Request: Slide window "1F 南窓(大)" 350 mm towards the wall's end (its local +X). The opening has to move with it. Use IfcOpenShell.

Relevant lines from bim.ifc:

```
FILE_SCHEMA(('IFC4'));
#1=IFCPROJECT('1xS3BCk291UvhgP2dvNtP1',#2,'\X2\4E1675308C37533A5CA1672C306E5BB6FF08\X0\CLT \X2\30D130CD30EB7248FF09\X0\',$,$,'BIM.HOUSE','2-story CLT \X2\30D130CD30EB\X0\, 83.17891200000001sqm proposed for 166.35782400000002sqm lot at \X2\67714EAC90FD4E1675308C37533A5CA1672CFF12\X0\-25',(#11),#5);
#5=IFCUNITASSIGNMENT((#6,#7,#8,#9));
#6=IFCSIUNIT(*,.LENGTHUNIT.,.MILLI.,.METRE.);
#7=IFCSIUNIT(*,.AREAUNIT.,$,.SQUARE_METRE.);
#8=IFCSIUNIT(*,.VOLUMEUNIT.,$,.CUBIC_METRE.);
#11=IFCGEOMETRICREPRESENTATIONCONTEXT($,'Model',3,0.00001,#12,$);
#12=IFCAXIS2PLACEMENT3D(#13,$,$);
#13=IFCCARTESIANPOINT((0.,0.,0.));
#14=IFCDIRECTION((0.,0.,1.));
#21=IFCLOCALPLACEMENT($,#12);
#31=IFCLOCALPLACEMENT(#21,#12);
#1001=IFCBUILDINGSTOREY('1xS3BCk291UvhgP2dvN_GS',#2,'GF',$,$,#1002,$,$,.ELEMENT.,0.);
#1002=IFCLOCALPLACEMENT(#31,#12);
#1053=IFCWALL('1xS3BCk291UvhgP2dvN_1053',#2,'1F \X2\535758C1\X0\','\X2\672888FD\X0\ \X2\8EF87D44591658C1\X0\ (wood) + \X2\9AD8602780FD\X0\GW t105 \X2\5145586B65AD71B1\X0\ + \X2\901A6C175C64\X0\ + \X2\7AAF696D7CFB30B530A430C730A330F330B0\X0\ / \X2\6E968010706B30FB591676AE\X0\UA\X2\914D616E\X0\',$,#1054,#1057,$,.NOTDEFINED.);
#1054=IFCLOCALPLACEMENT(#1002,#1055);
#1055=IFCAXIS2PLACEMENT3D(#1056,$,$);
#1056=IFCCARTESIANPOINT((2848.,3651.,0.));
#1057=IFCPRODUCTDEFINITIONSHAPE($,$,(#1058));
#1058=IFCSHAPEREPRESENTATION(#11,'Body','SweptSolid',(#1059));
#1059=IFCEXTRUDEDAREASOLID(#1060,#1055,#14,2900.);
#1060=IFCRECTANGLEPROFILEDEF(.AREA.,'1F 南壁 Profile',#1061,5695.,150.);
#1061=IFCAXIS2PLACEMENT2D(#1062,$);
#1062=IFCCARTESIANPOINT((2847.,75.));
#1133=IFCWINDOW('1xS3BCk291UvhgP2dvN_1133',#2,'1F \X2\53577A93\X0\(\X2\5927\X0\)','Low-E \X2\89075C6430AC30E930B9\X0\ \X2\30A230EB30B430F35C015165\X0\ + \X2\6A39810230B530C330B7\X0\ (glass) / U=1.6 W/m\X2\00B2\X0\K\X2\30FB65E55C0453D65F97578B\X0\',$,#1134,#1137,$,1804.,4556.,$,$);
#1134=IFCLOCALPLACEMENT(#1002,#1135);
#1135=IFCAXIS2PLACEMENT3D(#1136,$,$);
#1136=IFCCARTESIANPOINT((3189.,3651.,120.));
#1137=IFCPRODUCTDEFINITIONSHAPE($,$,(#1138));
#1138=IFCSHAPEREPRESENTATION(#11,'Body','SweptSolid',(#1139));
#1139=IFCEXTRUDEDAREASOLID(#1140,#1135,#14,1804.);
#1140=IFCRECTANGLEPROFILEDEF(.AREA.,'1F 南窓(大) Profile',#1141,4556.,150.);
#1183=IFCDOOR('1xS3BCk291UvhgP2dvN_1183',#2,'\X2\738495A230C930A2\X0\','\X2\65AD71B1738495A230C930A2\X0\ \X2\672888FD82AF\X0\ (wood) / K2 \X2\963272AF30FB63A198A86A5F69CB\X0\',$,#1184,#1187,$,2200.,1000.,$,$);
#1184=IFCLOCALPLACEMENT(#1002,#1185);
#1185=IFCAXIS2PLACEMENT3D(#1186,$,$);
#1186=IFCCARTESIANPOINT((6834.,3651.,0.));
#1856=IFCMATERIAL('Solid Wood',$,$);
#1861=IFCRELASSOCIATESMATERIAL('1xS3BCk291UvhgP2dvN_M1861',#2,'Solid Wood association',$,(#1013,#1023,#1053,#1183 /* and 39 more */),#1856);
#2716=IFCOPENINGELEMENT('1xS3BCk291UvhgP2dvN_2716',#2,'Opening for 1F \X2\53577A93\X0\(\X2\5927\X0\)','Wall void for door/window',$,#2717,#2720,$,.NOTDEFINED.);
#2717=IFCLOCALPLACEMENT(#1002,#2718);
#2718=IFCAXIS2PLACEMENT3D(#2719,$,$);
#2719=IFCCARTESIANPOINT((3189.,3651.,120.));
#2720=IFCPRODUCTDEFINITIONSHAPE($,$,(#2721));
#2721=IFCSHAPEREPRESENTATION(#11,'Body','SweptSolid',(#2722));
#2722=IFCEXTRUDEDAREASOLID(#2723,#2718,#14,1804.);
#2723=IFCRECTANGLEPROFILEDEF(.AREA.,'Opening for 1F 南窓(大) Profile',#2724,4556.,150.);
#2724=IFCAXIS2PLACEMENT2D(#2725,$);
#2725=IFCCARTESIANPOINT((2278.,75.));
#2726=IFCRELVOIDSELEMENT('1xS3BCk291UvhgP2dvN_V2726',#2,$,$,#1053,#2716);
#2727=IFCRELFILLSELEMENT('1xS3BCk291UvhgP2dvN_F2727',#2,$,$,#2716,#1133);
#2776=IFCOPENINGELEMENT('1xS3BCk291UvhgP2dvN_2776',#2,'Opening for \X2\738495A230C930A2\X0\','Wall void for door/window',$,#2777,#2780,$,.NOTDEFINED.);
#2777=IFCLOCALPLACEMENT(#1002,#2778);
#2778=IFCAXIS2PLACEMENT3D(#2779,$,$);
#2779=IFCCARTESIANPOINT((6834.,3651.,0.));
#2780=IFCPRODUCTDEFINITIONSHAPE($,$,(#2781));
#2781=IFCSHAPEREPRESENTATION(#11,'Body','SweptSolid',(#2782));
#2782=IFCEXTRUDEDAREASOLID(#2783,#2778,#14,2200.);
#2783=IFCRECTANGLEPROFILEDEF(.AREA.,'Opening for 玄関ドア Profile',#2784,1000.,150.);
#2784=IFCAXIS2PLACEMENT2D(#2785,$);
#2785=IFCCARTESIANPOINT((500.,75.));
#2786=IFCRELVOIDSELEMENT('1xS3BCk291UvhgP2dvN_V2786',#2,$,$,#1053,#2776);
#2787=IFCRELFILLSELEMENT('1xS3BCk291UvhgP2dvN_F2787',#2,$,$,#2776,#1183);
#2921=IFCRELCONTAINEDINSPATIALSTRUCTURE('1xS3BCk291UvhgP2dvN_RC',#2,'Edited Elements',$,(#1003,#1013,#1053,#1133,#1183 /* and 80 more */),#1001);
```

```python
import ifcopenshell
import ifcopenshell.api.geometry
import ifcopenshell.util.placement
import ifcopenshell.util.unit

model = ifcopenshell.open("bim.ifc")
unit_scale = ifcopenshell.util.unit.calculate_unit_scale(model)

window = model.by_guid("1xS3BCk291UvhgP2dvN_1133")
opening = window.FillsVoids[0].RelatingOpeningElement
wall = opening.VoidsElements[0].RelatingBuildingElement

wall_matrix = ifcopenshell.util.placement.get_local_placement(wall.ObjectPlacement)
shift = wall_matrix[:3, 0] * 0.35 / unit_scale
before = ifcopenshell.util.placement.get_local_placement(window.ObjectPlacement)[:3, 3].copy()

# The window is not placed relative to its opening, so move both.
for product in (opening, window):
    matrix = ifcopenshell.util.placement.get_local_placement(product.ObjectPlacement)
    matrix[:3, 3] += shift
    ifcopenshell.api.geometry.edit_object_placement(model, product=product, matrix=matrix, is_si=False)

after = ifcopenshell.util.placement.get_local_placement(window.ObjectPlacement)[:3, 3]
print("window moved by", (after - before).round(3) + 0.0)

model.write("bim_rev.ifc")
```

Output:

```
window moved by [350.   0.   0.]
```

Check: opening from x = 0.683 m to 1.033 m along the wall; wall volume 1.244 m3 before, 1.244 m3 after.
